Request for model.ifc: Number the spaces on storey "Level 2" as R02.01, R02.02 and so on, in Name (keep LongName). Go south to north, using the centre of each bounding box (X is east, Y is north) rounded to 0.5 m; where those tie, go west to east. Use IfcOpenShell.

First a look at what the model holds.

```python
import ifcopenshell
import ifcopenshell.util.element
import ifcopenshell.util.placement

model = ifcopenshell.open("model.ifc")
print(model.schema)
storey = next(s for s in model.by_type("IfcBuildingStorey") if s.Name == "Level 2")
spaces = [e for e in ifcopenshell.util.element.get_decomposition(storey) if e.is_a("IfcSpace")]
for e in sorted(spaces, key=lambda e: e.id()):
    origin = ifcopenshell.util.placement.get_local_placement(e.ObjectPlacement)[:3, 3]
    print(e.id(), e.Name, e.LongName, origin.round(2) + 0.0, sep=" | ")
```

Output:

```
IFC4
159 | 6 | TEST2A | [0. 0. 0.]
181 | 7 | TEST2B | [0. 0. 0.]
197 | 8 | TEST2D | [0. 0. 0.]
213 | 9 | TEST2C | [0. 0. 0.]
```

```python
import ifcopenshell
import ifcopenshell.geom
import ifcopenshell.util.element
import ifcopenshell.util.shape

model = ifcopenshell.open("model.ifc")
settings = ifcopenshell.geom.settings()
settings.set("use-world-coords", True)


def centre(element):
    shape = ifcopenshell.geom.create_shape(settings, element)
    return ifcopenshell.util.shape.get_bbox_centroid(shape.geometry)


storey = next(s for s in model.by_type("IfcBuildingStorey") if s.Name == "Level 2")
spaces = [e for e in ifcopenshell.util.element.get_decomposition(storey) if e.is_a("IfcSpace")]

# Insertion points can sit at a corner or the storey origin, so sort by the geometry (in metres).
centres = {e: centre(e) for e in spaces}
spaces.sort(key=lambda e: (round(centres[e][1] / 0.5), centres[e][0]))

for i, e in enumerate(spaces, start=1):
    number = f"R02.{i:02d}"
    e.Name = number
    print(e.id(), number)

model.write("model_v2.ifc")
```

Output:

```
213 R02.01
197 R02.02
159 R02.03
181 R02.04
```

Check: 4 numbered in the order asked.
